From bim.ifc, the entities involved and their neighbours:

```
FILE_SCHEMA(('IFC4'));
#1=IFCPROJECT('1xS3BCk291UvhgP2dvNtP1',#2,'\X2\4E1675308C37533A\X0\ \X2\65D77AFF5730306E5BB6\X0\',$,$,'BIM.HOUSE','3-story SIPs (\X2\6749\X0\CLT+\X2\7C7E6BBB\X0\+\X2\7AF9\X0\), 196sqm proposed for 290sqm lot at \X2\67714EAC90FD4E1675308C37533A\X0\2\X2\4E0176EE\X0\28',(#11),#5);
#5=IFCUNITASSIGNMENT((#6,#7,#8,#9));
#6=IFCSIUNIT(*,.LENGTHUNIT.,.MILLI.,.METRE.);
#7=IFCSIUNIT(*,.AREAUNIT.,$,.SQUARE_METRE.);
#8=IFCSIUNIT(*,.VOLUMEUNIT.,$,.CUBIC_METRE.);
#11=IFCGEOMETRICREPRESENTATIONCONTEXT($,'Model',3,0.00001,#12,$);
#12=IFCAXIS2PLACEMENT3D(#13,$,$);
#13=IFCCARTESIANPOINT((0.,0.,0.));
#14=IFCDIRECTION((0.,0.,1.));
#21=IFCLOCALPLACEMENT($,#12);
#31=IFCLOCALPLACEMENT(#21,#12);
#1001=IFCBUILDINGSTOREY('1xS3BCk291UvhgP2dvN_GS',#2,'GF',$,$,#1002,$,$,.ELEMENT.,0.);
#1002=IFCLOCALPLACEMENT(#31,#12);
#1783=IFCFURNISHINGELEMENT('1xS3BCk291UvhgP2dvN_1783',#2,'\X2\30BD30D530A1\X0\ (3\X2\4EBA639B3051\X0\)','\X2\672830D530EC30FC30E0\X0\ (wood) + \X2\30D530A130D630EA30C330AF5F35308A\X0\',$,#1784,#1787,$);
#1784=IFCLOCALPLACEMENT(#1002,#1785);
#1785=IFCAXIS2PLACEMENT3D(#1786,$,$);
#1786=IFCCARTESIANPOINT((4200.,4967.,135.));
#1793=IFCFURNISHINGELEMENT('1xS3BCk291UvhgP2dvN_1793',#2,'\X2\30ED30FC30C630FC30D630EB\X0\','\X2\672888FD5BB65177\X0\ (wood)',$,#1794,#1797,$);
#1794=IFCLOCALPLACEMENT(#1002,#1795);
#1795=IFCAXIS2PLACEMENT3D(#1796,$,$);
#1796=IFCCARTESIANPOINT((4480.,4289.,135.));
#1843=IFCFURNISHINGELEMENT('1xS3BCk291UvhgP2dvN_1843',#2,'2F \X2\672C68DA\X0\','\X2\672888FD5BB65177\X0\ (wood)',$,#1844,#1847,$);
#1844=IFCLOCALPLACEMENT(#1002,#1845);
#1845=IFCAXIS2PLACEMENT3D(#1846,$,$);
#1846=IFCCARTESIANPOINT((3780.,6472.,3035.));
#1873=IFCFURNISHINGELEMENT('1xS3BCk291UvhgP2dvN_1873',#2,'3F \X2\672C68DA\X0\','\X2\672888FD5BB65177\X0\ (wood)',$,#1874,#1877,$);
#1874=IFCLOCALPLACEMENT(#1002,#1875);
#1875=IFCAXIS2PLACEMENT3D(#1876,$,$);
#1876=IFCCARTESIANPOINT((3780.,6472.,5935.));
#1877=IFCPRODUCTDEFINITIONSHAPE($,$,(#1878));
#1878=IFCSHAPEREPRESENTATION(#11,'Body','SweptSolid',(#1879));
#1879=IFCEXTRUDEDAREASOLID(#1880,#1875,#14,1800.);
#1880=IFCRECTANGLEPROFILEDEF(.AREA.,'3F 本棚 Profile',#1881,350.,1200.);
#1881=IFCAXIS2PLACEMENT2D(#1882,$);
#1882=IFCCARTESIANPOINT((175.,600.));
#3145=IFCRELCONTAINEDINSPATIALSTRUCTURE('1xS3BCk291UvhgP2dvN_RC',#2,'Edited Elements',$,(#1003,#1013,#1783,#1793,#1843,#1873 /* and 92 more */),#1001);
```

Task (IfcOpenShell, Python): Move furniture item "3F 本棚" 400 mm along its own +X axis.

```python
import ifcopenshell
import ifcopenshell.api.geometry
import ifcopenshell.util.placement
import ifcopenshell.util.unit

model = ifcopenshell.open("bim.ifc")
unit_scale = ifcopenshell.util.unit.calculate_unit_scale(model)

item = model.by_guid("1xS3BCk291UvhgP2dvN_1873")
matrix = ifcopenshell.util.placement.get_local_placement(item.ObjectPlacement)
matrix[:3, 3] += matrix[:3, 0] * 0.4 / unit_scale
ifcopenshell.api.geometry.edit_object_placement(model, product=item, matrix=matrix, is_si=False)

print(ifcopenshell.util.placement.get_local_placement(item.ObjectPlacement).round(3) + 0.0)

model.write("bim_edited.ifc")
```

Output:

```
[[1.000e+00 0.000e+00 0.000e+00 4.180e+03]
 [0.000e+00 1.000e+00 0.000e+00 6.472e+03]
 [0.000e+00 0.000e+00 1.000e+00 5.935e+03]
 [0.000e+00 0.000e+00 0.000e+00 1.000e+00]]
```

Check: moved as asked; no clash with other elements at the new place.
